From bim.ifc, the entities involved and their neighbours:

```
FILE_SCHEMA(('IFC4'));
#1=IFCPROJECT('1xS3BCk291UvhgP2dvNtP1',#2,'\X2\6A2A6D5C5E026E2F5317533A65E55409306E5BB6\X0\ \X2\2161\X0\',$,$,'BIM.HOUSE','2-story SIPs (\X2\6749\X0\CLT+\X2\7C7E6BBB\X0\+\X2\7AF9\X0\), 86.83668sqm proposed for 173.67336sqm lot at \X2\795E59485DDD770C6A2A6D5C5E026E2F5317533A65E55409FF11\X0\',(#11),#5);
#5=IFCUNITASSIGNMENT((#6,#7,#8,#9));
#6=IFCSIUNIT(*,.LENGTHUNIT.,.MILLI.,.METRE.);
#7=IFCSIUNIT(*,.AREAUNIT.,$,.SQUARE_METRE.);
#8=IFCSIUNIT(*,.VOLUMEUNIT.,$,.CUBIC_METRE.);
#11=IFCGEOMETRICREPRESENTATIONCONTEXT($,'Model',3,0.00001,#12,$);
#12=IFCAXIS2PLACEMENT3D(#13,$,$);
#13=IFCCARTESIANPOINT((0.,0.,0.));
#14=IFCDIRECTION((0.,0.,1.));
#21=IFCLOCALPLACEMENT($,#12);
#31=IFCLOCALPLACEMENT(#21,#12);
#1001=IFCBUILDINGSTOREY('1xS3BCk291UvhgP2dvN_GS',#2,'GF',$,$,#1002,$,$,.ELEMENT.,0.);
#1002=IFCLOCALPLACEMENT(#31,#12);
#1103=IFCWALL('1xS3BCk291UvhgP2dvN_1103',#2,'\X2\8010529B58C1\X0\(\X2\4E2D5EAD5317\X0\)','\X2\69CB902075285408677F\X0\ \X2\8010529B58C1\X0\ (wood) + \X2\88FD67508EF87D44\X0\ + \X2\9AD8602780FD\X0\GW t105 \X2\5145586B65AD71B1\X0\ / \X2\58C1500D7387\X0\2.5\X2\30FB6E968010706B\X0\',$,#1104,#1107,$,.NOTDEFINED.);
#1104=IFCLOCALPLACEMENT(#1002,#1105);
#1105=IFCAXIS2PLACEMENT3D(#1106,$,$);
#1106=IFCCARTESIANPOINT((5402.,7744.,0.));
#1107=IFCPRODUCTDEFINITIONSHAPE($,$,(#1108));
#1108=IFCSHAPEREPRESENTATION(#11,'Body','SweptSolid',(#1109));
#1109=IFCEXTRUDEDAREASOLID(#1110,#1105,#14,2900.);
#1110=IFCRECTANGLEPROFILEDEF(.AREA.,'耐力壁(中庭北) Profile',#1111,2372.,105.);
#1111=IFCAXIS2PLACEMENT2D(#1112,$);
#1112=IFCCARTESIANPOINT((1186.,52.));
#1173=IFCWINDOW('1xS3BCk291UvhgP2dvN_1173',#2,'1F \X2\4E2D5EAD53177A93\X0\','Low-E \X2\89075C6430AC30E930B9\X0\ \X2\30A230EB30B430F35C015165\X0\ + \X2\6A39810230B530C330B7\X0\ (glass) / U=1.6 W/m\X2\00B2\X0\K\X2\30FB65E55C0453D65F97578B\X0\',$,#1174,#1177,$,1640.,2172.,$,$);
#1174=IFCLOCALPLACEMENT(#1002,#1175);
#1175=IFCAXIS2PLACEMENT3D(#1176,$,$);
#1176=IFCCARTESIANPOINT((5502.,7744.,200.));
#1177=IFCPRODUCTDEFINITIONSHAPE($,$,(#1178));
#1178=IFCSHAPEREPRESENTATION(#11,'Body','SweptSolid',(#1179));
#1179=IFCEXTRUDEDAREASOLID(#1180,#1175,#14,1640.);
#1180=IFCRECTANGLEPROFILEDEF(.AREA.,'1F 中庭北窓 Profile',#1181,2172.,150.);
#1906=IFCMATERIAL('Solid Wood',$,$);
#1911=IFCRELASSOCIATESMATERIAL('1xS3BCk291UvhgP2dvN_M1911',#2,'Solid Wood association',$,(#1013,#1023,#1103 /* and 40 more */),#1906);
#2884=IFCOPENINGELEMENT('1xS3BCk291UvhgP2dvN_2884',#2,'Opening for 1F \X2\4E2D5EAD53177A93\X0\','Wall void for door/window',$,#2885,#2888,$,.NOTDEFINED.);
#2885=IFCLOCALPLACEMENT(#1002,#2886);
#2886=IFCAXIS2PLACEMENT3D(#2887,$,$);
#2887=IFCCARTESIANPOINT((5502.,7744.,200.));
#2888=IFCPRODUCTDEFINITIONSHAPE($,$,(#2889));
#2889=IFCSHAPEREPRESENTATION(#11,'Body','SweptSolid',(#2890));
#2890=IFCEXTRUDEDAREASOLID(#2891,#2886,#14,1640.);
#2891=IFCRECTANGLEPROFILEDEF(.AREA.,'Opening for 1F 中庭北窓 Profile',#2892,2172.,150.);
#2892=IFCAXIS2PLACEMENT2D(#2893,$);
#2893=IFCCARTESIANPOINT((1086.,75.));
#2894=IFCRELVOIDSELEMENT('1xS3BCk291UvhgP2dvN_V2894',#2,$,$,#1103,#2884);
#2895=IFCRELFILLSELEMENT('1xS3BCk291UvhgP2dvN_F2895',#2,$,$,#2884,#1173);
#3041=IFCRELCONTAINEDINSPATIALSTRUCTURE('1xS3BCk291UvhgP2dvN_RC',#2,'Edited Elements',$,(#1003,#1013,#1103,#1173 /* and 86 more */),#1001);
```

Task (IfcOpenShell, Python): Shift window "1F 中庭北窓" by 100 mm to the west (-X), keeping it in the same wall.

```python
import ifcopenshell
import ifcopenshell.api.geometry
import ifcopenshell.util.placement
import ifcopenshell.util.unit

model = ifcopenshell.open("bim.ifc")
unit_scale = ifcopenshell.util.unit.calculate_unit_scale(model)

window = model.by_guid("1xS3BCk291UvhgP2dvN_1173")
opening = window.FillsVoids[0].RelatingOpeningElement
wall = opening.VoidsElements[0].RelatingBuildingElement

wall_matrix = ifcopenshell.util.placement.get_local_placement(wall.ObjectPlacement)
shift = wall_matrix[:3, 0] * -0.1 / unit_scale
before = ifcopenshell.util.placement.get_local_placement(window.ObjectPlacement)[:3, 3].copy()

# The window is not placed relative to its opening, so move both.
for product in (opening, window):
    matrix = ifcopenshell.util.placement.get_local_placement(product.ObjectPlacement)
    matrix[:3, 3] += shift
    ifcopenshell.api.geometry.edit_object_placement(model, product=product, matrix=matrix, is_si=False)

after = ifcopenshell.util.placement.get_local_placement(window.ObjectPlacement)[:3, 3]
print("window moved by", (after - before).round(3) + 0.0)

model.write("bim-out.ifc")
```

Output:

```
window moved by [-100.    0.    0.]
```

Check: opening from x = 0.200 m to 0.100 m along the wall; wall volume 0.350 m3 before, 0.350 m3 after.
